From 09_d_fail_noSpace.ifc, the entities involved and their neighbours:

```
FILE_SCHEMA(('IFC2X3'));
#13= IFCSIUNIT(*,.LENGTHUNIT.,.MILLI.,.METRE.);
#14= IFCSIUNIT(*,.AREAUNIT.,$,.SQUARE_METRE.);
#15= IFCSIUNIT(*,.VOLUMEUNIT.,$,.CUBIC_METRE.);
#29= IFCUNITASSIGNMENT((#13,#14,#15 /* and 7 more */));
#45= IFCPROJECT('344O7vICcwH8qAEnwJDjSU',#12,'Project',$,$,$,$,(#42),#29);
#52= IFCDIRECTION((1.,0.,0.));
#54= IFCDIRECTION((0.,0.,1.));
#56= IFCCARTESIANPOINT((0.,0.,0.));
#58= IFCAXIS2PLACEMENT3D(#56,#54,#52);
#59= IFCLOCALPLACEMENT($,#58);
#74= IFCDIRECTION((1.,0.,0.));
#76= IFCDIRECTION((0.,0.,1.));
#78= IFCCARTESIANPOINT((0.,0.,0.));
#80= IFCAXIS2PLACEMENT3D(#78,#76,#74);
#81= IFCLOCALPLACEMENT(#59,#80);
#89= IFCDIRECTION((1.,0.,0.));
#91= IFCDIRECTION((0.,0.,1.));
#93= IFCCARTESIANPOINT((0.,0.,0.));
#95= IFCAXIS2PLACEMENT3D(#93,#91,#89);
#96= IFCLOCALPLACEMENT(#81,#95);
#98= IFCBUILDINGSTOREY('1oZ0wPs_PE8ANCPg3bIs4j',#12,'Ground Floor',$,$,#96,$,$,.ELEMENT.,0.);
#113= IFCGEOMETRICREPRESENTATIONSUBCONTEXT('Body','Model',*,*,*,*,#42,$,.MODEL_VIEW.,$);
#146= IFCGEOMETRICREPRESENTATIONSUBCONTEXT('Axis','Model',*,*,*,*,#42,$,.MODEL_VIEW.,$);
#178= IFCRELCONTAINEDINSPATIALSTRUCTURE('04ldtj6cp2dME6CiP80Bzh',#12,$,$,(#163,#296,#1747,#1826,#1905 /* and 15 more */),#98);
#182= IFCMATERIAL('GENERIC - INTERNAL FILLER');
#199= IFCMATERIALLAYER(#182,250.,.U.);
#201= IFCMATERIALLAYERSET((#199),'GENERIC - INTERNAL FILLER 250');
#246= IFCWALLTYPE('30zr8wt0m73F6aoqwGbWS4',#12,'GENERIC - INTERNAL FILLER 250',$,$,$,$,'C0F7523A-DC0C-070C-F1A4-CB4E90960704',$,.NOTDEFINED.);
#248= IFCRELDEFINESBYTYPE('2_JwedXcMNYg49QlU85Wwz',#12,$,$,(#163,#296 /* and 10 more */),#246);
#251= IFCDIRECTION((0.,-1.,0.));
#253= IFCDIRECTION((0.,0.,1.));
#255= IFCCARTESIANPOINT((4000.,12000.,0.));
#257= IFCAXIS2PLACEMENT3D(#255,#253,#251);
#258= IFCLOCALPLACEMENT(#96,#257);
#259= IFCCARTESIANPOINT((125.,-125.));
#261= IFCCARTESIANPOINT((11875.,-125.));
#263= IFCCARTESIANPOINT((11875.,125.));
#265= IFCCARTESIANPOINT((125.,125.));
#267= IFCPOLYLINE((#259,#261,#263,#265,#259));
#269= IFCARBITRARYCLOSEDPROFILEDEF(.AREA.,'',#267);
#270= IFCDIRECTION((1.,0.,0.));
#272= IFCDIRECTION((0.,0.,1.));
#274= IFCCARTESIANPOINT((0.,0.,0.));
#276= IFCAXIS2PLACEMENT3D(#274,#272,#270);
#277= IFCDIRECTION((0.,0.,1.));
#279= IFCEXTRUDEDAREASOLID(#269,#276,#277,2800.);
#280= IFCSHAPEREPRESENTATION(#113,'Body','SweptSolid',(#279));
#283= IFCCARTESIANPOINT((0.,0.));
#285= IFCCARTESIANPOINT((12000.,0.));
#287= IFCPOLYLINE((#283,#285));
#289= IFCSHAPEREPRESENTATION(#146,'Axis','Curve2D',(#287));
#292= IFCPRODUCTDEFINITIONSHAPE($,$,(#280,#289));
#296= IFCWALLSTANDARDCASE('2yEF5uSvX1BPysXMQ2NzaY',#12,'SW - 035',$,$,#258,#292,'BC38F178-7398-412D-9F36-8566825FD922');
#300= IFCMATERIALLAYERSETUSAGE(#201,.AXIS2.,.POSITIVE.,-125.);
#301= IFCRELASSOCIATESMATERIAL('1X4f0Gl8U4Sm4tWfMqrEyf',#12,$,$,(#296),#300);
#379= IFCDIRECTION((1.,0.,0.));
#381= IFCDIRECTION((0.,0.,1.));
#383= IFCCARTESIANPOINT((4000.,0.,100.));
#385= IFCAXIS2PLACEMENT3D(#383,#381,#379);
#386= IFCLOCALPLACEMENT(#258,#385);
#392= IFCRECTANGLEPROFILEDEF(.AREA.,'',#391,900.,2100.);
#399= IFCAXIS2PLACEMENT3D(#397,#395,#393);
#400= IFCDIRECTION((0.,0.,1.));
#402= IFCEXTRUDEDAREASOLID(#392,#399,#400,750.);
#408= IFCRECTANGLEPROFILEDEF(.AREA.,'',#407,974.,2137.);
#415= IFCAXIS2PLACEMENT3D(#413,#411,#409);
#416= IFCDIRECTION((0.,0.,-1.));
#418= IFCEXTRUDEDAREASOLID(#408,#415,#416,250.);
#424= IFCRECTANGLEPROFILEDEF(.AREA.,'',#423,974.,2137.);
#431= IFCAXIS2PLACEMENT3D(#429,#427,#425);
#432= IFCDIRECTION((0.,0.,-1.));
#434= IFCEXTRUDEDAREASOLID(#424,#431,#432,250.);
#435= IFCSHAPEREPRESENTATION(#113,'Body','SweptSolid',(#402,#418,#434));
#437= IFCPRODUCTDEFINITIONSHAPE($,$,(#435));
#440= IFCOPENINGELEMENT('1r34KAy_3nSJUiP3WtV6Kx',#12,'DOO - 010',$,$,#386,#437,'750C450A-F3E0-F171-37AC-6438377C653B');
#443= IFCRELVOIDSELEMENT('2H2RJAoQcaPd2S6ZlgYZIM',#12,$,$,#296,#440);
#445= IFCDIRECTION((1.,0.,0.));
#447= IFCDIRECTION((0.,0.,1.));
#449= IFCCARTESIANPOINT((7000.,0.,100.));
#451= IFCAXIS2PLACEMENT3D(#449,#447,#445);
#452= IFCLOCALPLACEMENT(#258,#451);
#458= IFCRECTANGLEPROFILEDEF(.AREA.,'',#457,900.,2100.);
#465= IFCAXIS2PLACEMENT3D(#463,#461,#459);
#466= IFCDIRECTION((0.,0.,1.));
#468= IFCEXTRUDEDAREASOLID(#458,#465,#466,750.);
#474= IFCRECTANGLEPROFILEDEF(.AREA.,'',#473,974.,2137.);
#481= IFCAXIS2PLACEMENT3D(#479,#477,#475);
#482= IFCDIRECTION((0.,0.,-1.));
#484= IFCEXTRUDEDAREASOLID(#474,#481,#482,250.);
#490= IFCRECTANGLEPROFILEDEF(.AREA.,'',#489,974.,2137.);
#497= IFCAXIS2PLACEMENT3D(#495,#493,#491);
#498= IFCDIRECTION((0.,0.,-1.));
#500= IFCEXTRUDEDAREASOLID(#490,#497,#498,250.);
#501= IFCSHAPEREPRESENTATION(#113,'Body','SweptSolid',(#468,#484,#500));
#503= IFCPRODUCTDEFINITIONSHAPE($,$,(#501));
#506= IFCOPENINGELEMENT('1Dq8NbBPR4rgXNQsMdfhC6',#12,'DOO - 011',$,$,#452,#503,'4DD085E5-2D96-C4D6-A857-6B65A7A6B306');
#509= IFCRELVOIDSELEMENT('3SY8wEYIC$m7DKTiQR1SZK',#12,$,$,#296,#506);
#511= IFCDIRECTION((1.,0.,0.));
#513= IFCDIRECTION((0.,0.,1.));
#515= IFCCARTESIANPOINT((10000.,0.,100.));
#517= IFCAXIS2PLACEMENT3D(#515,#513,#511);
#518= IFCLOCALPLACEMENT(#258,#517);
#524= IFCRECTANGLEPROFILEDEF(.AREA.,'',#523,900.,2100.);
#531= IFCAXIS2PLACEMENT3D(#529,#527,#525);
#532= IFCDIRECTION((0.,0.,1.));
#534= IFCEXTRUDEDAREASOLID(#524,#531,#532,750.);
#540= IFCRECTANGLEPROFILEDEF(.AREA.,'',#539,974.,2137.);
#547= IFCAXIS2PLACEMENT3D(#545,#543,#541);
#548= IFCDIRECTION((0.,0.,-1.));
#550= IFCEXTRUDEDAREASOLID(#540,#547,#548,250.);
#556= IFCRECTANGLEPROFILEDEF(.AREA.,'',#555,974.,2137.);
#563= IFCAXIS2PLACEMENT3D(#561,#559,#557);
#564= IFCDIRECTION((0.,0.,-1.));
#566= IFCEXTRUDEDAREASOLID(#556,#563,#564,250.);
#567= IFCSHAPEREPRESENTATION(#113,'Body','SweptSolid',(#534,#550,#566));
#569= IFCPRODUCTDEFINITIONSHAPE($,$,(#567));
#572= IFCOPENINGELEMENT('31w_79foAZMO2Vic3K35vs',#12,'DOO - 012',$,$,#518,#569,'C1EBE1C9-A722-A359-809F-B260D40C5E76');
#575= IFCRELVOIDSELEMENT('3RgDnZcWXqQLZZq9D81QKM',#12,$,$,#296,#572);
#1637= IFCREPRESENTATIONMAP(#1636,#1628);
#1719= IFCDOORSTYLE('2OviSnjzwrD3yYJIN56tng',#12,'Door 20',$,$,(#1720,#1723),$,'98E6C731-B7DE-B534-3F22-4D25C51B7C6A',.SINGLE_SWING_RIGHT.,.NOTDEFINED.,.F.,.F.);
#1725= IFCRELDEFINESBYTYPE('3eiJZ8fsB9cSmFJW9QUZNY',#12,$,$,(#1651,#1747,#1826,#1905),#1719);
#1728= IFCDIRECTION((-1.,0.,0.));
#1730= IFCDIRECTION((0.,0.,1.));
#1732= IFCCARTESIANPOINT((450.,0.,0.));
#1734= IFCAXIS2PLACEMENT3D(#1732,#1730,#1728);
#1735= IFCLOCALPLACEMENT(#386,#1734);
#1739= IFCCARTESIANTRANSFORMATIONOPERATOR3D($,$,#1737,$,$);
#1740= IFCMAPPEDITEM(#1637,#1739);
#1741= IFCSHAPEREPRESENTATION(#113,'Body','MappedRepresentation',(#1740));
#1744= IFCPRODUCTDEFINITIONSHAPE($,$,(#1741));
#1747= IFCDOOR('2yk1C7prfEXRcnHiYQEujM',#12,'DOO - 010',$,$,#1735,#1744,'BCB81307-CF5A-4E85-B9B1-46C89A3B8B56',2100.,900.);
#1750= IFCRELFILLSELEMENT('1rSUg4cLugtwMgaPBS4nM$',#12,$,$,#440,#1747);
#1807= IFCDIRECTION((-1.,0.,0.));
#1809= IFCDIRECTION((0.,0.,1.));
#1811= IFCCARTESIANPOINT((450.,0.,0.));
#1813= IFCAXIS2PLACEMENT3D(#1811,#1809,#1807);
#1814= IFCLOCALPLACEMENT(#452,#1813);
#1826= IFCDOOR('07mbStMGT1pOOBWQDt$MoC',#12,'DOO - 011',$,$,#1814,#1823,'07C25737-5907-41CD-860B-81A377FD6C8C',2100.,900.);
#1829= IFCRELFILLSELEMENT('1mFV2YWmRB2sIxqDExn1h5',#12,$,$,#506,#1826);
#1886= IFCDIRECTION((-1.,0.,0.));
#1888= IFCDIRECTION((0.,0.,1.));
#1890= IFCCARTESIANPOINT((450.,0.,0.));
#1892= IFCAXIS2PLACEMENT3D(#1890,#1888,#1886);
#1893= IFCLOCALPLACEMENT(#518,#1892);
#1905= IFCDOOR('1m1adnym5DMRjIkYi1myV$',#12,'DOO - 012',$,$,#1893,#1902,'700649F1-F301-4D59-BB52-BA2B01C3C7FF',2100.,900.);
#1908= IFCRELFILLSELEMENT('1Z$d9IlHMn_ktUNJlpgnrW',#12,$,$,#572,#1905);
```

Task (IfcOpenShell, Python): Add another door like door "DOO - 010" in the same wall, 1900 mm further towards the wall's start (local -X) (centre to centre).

```python
import ifcopenshell
import ifcopenshell.api.feature
import ifcopenshell.api.geometry
import ifcopenshell.api.root
import ifcopenshell.geom
import ifcopenshell.util.element
import ifcopenshell.util.placement
import ifcopenshell.util.shape
import ifcopenshell.util.unit

model = ifcopenshell.open("09_d_fail_noSpace.ifc")
unit_scale = ifcopenshell.util.unit.calculate_unit_scale(model)
settings = ifcopenshell.geom.settings()


def volume(element):
    """Net volume in cubic metres, openings subtracted."""
    shape = ifcopenshell.geom.create_shape(settings, element)
    return ifcopenshell.util.shape.get_volume(shape.geometry)


def reuse_history(source, copy):
    """copy_class also copies each property set's owner history, people and application; keep the originals."""
    for rel in copy.IsDefinedBy:
        if rel.is_a("IfcRelDefinesByProperties") and (history := rel.RelatingPropertyDefinition.OwnerHistory):
            rel.RelatingPropertyDefinition.OwnerHistory = source.OwnerHistory
            ifcopenshell.util.element.remove_deep2(model, history)


door = model.by_guid("2yk1C7prfEXRcnHiYQEujM")
opening = door.FillsVoids[0].RelatingOpeningElement
wall = opening.VoidsElements[0].RelatingBuildingElement
before = volume(wall)
shift = ifcopenshell.util.placement.get_local_placement(wall.ObjectPlacement)[:3, 0] * -1.9 / unit_scale

# copy_class copies the void relationship, type, container and properties, but no geometry.
new_opening = ifcopenshell.api.root.copy_class(model, product=opening)
new_opening.Representation = ifcopenshell.util.element.copy_deep(
    model, opening.Representation, exclude=["IfcGeometricRepresentationContext", "IfcRepresentationMap"]
)
new_opening.Tag = None
new_door = ifcopenshell.api.root.copy_class(model, product=door)
new_door.Representation = ifcopenshell.util.element.copy_deep(
    model, door.Representation, exclude=["IfcGeometricRepresentationContext", "IfcRepresentationMap"]
)
new_door.Tag = None
reuse_history(door, new_door)
fills = ifcopenshell.api.feature.add_filling(model, opening=new_opening, element=new_door)
fills.OwnerHistory = new_door.OwnerHistory  # required in IFC2X3

for old, new in ((opening, new_opening), (door, new_door)):
    matrix = ifcopenshell.util.placement.get_local_placement(old.ObjectPlacement)
    matrix[:3, 3] += shift
    ifcopenshell.api.geometry.edit_object_placement(model, product=new, matrix=matrix, is_si=False)

after = volume(wall)

print(f"wall volume {before:.3f} -> {after:.3f} m3")

model.write("09_d_fail_noSpace-out.ifc")
```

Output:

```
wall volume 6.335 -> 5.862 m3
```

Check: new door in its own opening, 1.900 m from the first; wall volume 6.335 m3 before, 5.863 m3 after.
